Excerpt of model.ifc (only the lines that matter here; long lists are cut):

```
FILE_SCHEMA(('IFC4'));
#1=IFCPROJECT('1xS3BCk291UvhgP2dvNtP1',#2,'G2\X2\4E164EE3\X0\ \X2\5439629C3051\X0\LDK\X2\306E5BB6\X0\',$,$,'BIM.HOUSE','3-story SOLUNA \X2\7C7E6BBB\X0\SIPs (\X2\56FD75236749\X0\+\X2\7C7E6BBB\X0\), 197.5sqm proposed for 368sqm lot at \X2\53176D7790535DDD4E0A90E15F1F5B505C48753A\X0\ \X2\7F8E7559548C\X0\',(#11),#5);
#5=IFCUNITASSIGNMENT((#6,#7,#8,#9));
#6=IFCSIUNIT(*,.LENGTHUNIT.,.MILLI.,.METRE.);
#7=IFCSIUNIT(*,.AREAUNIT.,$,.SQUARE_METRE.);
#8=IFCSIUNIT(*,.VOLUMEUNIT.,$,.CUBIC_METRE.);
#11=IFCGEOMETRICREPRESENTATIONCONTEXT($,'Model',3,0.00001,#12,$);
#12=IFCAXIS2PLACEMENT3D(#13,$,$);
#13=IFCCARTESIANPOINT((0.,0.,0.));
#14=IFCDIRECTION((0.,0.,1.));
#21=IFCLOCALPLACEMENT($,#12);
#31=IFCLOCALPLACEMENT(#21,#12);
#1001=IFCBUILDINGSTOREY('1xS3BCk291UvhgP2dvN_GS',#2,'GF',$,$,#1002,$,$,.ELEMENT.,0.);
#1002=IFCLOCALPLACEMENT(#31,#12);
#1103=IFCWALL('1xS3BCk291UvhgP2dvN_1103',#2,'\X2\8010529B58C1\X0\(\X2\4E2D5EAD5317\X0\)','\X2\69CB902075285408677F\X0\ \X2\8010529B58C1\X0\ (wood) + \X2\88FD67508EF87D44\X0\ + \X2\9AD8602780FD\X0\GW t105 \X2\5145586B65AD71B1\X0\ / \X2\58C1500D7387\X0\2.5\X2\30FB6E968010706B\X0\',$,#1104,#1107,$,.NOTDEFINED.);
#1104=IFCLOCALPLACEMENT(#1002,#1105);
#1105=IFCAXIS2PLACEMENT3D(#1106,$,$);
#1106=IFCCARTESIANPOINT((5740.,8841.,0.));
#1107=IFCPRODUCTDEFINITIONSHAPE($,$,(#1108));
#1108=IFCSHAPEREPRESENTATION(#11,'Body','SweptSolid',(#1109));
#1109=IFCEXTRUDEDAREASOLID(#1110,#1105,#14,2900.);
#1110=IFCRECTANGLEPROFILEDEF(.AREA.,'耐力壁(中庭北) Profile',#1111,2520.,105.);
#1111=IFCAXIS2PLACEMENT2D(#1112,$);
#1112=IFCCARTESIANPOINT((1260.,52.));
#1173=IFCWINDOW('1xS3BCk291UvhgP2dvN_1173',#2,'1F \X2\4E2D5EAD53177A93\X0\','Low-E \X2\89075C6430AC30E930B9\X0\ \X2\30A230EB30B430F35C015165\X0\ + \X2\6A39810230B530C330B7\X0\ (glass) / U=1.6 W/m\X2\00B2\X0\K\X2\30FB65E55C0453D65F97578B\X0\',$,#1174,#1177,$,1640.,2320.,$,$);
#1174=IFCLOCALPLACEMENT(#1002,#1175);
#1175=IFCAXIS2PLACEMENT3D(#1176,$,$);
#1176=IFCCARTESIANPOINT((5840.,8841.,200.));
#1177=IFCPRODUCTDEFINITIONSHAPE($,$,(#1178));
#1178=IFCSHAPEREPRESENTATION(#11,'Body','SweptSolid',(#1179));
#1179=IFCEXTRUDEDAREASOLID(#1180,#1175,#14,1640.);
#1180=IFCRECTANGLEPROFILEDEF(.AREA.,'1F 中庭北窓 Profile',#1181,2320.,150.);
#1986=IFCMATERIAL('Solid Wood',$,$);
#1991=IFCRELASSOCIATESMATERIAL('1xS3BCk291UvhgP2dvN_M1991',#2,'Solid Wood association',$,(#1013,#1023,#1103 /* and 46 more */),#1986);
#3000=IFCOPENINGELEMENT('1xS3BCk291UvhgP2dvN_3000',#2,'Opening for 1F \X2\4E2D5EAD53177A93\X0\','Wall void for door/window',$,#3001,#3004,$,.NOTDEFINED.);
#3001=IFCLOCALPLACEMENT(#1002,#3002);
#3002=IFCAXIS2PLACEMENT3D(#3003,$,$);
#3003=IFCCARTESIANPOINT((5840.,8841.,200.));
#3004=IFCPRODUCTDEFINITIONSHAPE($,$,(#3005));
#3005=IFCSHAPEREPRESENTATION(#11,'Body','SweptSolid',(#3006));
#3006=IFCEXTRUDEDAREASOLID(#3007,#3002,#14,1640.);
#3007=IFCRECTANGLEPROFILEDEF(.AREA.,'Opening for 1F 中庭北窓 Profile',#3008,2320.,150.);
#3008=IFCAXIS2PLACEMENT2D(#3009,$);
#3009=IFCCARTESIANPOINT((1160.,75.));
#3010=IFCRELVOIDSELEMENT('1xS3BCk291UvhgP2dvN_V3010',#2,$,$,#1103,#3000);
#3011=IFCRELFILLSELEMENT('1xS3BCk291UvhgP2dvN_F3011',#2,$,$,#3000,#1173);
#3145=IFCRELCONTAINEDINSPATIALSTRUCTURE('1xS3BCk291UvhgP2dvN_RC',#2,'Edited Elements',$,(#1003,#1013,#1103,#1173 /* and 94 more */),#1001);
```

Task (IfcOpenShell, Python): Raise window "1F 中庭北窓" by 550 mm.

```python
import numpy as np
import ifcopenshell
import ifcopenshell.api.geometry
import ifcopenshell.util.placement
import ifcopenshell.util.unit

model = ifcopenshell.open("model.ifc")
unit_scale = ifcopenshell.util.unit.calculate_unit_scale(model)

window = model.by_id(1173)
opening = window.FillsVoids[0].RelatingOpeningElement
dz = 0.55 / unit_scale

shift = np.array([0.0, 0.0, dz])
# The window is not placed relative to its opening, so move both.
for product in (opening, window):
    matrix = ifcopenshell.util.placement.get_local_placement(product.ObjectPlacement)
    matrix[:3, 3] += shift
    ifcopenshell.api.geometry.edit_object_placement(model, product=product, matrix=matrix, is_si=False)

print(f"moved by {dz * unit_scale:+.3f} m")

model.write("model_updated.ifc")
```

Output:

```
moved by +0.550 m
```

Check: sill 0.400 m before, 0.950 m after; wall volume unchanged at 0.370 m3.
